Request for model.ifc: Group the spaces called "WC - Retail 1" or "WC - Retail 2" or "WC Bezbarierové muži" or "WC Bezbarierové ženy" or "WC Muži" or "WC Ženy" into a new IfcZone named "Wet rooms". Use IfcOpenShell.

First a look at what the model holds.

```python
import ifcopenshell

model = ifcopenshell.open("model.ifc")
print(model.schema)
seen = {}
for space in model.by_type("IfcSpace"):
    seen[space.LongName] = seen.get(space.LongName, 0) + 1
for name, count in sorted(seen.items(), key=str):
    print(count, "x", name)
print("zones:", [z.Name for z in model.by_type("IfcZone")][:20])
```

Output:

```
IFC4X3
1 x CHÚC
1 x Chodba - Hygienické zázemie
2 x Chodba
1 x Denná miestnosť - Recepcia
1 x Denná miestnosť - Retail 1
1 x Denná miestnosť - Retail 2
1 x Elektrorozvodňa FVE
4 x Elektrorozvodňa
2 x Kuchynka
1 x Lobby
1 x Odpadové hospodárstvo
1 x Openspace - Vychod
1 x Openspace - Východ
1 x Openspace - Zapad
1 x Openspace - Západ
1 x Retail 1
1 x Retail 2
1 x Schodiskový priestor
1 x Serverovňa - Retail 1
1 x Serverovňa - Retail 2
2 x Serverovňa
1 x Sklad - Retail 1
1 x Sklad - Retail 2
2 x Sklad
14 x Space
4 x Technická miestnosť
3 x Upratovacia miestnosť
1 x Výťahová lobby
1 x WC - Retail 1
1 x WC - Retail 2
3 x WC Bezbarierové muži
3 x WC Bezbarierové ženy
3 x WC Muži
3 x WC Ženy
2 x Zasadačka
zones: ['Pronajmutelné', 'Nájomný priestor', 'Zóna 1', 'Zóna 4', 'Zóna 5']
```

```python
import ifcopenshell
import ifcopenshell.api.group
import ifcopenshell.api.root

model = ifcopenshell.open("model.ifc")

names = {"WC - Retail 1", "WC - Retail 2", "WC Bezbarierové muži", "WC Bezbarierové ženy", "WC Muži", "WC Ženy"}
spaces = [s for s in model.by_type("IfcSpace") if s.LongName in names]

zone = ifcopenshell.api.root.create_entity(model, ifc_class="IfcZone", name="Wet rooms")
ifcopenshell.api.group.assign_group(model, products=spaces, group=zone)
print(len(spaces), "spaces in", zone.Name)

model.write("model_edited.ifc")
```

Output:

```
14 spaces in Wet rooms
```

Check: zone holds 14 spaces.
